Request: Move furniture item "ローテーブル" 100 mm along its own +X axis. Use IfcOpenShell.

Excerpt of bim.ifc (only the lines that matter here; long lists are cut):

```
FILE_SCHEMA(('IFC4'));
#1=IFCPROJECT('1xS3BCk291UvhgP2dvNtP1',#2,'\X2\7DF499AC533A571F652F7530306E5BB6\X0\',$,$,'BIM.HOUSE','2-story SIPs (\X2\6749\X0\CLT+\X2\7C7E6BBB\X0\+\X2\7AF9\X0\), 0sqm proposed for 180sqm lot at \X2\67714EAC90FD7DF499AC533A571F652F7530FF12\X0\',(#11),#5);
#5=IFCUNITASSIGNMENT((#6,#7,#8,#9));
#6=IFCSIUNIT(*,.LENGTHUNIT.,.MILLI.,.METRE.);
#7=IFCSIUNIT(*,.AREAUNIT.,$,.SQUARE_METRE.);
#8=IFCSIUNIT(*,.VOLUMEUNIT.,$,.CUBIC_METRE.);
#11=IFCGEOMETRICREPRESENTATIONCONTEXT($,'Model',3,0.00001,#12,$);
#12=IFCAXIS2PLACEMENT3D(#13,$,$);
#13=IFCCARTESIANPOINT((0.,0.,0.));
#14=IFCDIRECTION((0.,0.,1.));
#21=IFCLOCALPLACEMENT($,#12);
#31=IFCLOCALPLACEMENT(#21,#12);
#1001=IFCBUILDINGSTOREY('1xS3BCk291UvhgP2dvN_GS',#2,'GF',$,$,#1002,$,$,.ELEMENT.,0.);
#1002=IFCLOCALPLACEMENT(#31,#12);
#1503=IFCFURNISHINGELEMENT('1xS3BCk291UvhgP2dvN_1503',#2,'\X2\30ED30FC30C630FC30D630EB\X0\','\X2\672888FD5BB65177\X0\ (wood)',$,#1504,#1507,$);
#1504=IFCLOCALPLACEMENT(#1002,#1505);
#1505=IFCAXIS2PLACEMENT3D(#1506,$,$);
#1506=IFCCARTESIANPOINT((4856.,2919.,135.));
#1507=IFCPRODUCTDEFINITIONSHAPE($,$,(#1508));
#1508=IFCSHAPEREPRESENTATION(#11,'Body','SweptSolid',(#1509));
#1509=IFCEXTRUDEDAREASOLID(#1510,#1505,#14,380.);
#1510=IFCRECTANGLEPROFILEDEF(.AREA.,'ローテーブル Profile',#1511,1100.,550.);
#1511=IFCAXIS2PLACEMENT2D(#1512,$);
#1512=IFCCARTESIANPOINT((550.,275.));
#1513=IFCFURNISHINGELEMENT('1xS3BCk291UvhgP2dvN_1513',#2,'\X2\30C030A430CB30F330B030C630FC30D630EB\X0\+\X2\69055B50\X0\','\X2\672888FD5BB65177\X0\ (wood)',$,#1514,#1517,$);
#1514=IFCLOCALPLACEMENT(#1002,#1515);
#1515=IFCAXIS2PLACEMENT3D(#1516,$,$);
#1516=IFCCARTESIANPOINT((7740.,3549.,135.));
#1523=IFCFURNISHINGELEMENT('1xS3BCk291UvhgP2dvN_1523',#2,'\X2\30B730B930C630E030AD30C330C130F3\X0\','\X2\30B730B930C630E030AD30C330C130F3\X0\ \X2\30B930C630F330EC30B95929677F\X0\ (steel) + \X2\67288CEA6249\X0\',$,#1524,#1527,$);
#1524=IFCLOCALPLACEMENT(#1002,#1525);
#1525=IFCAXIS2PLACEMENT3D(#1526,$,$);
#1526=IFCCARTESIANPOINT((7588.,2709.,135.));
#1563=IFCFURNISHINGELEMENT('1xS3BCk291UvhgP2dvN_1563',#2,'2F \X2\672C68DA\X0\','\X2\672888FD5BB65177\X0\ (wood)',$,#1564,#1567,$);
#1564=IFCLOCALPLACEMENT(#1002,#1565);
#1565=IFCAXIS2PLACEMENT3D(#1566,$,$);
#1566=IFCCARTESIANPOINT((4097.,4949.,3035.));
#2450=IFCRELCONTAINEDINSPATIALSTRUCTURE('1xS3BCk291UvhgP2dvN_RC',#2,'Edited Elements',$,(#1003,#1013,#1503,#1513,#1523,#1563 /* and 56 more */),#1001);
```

```python
import ifcopenshell
import ifcopenshell.api.geometry
import ifcopenshell.util.placement

model = ifcopenshell.open("bim.ifc")

item = model.by_guid("1xS3BCk291UvhgP2dvN_1503")
matrix = ifcopenshell.util.placement.get_local_placement(item.ObjectPlacement)
matrix[:3, 3] += matrix[:3, 0] * 100.0
ifcopenshell.api.geometry.edit_object_placement(model, product=item, matrix=matrix, is_si=False)

print(ifcopenshell.util.placement.get_local_placement(item.ObjectPlacement).round(3) + 0.0)

model.write("bim_edited.ifc")
```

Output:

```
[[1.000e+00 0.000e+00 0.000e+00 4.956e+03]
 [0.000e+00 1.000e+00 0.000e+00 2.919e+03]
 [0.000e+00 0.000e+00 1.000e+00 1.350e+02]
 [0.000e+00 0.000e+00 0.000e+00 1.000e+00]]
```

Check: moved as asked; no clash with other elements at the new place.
